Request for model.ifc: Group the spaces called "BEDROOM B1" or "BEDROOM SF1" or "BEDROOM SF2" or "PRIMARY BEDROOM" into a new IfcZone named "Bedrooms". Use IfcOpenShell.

First a look at what the model holds.

```python
import ifcopenshell

model = ifcopenshell.open("model.ifc")
print(model.schema)
seen = {}
for space in model.by_type("IfcSpace"):
    seen[space.LongName] = seen.get(space.LongName, 0) + 1
for name, count in sorted(seen.items(), key=str):
    print(count, "x", name)
print("zones:", [z.Name for z in model.by_type("IfcZone")][:20])
```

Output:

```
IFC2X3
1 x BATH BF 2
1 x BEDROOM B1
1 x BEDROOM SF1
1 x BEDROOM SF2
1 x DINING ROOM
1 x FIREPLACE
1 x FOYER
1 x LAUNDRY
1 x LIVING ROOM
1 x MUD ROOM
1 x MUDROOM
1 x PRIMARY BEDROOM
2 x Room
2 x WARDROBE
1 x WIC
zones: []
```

```python
import ifcopenshell
import ifcopenshell.api.group
import ifcopenshell.api.root

model = ifcopenshell.open("model.ifc")

names = {"BEDROOM B1", "BEDROOM SF1", "BEDROOM SF2", "PRIMARY BEDROOM"}
spaces = [s for s in model.by_type("IfcSpace") if s.LongName in names]

zone = ifcopenshell.api.root.create_entity(model, ifc_class="IfcZone", name="Bedrooms")
ifcopenshell.api.group.assign_group(model, products=spaces, group=zone)
print(len(spaces), "spaces in", zone.Name)

model.write("model_v2.ifc")
```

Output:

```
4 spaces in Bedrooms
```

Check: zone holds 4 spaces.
